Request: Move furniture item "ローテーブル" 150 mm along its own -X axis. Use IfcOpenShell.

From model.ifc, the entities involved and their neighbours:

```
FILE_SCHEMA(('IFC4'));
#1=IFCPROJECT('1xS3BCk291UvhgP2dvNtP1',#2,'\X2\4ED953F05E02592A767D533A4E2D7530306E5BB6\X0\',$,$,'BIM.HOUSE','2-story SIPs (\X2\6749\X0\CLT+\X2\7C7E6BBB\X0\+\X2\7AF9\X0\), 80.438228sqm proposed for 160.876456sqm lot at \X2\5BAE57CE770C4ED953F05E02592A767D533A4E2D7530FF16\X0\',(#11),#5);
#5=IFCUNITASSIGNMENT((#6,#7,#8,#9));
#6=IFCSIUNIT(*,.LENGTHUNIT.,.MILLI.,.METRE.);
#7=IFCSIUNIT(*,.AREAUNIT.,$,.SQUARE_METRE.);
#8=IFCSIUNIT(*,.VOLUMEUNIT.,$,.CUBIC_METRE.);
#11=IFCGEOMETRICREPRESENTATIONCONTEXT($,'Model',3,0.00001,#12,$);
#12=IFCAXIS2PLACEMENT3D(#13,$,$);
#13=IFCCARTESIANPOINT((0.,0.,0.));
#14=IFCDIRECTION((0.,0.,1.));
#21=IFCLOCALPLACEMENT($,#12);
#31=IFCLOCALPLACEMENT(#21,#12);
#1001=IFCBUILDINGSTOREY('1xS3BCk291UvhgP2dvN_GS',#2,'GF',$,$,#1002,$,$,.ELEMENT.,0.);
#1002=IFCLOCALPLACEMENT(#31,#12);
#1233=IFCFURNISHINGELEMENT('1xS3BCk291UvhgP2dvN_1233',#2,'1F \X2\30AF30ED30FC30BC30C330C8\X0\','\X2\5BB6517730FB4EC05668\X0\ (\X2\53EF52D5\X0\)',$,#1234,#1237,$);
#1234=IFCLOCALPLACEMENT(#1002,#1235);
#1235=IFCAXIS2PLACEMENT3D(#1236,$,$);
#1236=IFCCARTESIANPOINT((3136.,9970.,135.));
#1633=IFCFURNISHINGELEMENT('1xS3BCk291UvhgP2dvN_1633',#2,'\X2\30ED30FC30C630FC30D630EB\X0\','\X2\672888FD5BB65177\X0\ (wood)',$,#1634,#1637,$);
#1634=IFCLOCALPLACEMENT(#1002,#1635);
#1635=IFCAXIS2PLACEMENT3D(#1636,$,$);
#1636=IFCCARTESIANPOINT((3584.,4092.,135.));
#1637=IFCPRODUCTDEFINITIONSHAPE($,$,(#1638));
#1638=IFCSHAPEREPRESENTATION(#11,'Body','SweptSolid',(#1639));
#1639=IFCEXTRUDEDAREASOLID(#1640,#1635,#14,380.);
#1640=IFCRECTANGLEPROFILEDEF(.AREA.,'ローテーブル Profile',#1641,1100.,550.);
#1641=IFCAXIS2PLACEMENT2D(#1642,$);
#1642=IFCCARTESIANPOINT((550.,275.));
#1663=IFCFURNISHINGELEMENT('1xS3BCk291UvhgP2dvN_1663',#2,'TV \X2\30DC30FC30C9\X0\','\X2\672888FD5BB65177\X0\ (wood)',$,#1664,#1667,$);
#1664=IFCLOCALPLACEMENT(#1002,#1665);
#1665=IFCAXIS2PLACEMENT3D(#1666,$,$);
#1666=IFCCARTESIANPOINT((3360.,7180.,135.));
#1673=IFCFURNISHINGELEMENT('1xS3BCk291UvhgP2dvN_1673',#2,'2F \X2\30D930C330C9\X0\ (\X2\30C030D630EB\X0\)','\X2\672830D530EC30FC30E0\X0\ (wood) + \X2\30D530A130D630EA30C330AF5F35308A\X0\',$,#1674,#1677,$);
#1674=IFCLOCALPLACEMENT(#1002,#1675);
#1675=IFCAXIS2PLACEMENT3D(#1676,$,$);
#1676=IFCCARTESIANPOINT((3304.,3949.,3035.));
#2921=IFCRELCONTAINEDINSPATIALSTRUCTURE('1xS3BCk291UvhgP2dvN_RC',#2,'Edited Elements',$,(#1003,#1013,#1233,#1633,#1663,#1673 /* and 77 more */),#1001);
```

```python
import ifcopenshell
import ifcopenshell.api.geometry
import ifcopenshell.util.placement

model = ifcopenshell.open("model.ifc")

item = model.by_id(1633)
matrix = ifcopenshell.util.placement.get_local_placement(item.ObjectPlacement)
matrix[:3, 3] -= matrix[:3, 0] * 150.0
ifcopenshell.api.geometry.edit_object_placement(model, product=item, matrix=matrix, is_si=False)

print(ifcopenshell.util.placement.get_local_placement(item.ObjectPlacement).round(3) + 0.0)

model.write("model-out.ifc")
```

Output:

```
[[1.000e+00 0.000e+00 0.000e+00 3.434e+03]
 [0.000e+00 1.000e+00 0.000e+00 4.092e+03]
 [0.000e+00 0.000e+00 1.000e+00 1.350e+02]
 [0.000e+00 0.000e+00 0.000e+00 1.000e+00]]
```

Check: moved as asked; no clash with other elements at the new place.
